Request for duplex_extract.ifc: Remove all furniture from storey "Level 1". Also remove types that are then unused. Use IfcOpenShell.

First a look at what the model holds.

```python
import ifcopenshell
import ifcopenshell.util.element

model = ifcopenshell.open("duplex_extract.ifc")
print(model.schema)
storey = next(s for s in model.by_type("IfcBuildingStorey") if s.Name == "Level 1")
furniture = [e for e in ifcopenshell.util.element.get_decomposition(storey) if e.is_a("IfcFurnishingElement")]
seen = {}
for e in furniture:
    element_type = ifcopenshell.util.element.get_type(e)
    name = element_type.Name if element_type not in (None, e) else None
    seen[name] = seen.get(name, 0) + 1
for name, count in sorted(seen.items(), key=str):
    print(count, "x", name)
```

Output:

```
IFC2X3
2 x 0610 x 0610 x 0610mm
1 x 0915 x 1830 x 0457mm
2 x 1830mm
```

```python
import ifcopenshell
import ifcopenshell.api.root
import ifcopenshell.util.element

model = ifcopenshell.open("duplex_extract.ifc")

storey = next(s for s in model.by_type("IfcBuildingStorey") if s.Name == "Level 1")
furniture = [e for e in ifcopenshell.util.element.get_decomposition(storey) if e.is_a("IfcFurnishingElement")]
types = {ifcopenshell.util.element.get_type(e) for e in furniture} - {None, *furniture}

for e in furniture:
    ifcopenshell.api.root.remove_product(model, product=e)
print(len(furniture), "removed")

unused = [t for t in types if not ifcopenshell.util.element.get_types(t)]
for t in unused:
    ifcopenshell.api.root.remove_product(model, product=t)
print(len(unused), "unused types removed")

model.write("duplex_extract_rev.ifc")
```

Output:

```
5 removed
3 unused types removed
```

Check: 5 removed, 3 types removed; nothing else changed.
